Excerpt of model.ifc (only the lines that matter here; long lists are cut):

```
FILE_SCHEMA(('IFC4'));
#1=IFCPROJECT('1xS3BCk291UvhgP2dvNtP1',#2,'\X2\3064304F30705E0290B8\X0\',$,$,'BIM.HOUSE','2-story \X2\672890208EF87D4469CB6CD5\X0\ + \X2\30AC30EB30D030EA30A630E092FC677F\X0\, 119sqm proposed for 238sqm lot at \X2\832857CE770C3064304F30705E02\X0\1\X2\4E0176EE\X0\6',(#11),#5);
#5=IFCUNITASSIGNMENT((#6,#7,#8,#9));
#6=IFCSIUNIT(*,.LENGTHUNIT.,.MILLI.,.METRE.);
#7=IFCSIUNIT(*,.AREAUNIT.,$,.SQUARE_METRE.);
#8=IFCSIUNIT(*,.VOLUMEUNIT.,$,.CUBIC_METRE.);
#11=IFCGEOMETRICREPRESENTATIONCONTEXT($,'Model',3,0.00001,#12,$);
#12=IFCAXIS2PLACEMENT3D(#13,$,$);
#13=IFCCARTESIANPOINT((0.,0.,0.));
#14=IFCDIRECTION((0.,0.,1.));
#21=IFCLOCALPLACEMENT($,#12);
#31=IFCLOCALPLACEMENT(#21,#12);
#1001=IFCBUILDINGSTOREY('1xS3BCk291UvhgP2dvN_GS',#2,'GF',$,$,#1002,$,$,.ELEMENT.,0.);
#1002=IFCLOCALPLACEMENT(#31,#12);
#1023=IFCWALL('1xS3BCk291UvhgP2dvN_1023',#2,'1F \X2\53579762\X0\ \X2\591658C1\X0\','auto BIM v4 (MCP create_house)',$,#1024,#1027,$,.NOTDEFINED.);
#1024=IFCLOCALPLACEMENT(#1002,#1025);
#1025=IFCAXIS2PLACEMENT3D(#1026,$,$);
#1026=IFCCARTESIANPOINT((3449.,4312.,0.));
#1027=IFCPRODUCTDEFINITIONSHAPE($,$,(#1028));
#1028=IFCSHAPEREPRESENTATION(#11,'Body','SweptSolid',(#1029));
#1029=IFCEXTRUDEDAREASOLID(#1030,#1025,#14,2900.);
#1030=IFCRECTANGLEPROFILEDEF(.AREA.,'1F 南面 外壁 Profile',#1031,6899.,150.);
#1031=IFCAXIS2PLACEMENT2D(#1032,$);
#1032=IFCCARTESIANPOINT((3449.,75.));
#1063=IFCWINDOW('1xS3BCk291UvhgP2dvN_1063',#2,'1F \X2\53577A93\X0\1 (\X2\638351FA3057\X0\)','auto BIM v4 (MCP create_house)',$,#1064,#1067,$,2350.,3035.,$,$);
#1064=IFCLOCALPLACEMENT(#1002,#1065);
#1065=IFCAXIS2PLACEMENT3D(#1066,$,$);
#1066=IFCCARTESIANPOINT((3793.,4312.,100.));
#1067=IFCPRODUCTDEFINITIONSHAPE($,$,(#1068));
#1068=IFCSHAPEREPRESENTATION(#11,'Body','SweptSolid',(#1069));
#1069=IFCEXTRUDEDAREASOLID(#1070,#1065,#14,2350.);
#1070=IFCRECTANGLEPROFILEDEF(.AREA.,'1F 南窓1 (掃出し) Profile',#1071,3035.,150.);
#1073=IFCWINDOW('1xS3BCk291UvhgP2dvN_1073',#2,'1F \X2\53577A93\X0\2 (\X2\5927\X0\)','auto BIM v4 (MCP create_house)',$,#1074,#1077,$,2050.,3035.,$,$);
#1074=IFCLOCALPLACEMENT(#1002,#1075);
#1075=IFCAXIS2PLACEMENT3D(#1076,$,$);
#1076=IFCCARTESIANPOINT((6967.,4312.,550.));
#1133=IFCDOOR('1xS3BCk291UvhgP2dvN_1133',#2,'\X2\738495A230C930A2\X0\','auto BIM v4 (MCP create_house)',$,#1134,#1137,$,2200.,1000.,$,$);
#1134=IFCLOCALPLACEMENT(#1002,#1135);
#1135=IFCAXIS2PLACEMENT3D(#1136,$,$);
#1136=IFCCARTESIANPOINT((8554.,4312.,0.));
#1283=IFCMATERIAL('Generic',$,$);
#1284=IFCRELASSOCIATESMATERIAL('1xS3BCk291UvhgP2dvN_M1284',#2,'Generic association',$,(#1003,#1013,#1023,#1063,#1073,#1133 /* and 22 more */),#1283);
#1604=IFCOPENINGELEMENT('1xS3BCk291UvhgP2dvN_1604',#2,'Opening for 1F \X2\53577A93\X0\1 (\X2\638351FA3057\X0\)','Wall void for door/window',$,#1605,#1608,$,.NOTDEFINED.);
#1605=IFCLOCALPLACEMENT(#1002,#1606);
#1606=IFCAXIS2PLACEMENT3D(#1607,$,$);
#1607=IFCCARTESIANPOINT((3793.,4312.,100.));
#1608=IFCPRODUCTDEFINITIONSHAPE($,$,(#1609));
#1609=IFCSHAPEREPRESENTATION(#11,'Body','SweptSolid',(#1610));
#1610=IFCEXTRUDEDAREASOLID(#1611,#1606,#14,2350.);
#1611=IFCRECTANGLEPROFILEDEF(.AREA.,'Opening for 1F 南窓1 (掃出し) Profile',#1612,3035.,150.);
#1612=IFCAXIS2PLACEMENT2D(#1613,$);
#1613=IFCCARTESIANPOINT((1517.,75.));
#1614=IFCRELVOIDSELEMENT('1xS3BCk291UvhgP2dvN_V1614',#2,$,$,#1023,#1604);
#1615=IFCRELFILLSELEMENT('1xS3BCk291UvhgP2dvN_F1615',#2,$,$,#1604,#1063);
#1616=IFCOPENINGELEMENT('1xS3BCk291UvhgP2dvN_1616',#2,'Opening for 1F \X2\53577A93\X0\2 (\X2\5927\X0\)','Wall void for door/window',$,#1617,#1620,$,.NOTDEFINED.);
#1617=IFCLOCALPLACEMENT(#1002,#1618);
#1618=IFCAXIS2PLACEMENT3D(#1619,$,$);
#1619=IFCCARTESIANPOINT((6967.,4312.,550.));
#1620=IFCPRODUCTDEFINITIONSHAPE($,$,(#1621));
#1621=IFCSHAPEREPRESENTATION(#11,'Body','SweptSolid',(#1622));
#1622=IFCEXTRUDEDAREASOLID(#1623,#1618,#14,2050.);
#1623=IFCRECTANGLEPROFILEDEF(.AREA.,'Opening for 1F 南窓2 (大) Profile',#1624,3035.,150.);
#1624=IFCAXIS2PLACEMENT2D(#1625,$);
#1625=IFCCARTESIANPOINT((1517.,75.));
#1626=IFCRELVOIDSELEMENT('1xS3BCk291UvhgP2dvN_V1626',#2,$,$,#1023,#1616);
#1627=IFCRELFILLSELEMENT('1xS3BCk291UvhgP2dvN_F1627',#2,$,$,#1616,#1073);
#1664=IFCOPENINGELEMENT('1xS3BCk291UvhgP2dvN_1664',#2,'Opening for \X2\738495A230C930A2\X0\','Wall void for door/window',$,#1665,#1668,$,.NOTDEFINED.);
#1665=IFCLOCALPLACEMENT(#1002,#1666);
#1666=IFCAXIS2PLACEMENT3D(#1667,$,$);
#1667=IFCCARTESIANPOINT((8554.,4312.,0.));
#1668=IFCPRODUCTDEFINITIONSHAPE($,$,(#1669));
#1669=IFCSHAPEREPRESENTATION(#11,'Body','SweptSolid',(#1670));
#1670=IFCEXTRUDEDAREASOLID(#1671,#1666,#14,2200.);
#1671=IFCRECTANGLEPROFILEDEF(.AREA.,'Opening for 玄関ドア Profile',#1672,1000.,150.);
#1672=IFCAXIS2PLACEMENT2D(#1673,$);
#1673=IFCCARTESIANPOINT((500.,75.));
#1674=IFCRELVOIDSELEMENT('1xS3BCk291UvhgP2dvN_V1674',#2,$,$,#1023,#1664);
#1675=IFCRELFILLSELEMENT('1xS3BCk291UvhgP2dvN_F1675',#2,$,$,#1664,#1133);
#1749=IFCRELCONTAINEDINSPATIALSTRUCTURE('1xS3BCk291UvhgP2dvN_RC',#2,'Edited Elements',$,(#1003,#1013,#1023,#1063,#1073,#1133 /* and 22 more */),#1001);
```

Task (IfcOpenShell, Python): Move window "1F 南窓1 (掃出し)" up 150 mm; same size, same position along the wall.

```python
import numpy as np
import ifcopenshell
import ifcopenshell.api.geometry
import ifcopenshell.util.placement
import ifcopenshell.util.unit

model = ifcopenshell.open("model.ifc")
unit_scale = ifcopenshell.util.unit.calculate_unit_scale(model)

window = model.by_guid("1xS3BCk291UvhgP2dvN_1063")
opening = window.FillsVoids[0].RelatingOpeningElement
dz = 150.0

shift = np.array([0.0, 0.0, dz])
# The window is not placed relative to its opening, so move both.
for product in (opening, window):
    matrix = ifcopenshell.util.placement.get_local_placement(product.ObjectPlacement)
    matrix[:3, 3] += shift
    ifcopenshell.api.geometry.edit_object_placement(model, product=product, matrix=matrix, is_si=False)

print(f"moved by {dz * unit_scale:+.3f} m")

model.write("model_rev.ifc")
```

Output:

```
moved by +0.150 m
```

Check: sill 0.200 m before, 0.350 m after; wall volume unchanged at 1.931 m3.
